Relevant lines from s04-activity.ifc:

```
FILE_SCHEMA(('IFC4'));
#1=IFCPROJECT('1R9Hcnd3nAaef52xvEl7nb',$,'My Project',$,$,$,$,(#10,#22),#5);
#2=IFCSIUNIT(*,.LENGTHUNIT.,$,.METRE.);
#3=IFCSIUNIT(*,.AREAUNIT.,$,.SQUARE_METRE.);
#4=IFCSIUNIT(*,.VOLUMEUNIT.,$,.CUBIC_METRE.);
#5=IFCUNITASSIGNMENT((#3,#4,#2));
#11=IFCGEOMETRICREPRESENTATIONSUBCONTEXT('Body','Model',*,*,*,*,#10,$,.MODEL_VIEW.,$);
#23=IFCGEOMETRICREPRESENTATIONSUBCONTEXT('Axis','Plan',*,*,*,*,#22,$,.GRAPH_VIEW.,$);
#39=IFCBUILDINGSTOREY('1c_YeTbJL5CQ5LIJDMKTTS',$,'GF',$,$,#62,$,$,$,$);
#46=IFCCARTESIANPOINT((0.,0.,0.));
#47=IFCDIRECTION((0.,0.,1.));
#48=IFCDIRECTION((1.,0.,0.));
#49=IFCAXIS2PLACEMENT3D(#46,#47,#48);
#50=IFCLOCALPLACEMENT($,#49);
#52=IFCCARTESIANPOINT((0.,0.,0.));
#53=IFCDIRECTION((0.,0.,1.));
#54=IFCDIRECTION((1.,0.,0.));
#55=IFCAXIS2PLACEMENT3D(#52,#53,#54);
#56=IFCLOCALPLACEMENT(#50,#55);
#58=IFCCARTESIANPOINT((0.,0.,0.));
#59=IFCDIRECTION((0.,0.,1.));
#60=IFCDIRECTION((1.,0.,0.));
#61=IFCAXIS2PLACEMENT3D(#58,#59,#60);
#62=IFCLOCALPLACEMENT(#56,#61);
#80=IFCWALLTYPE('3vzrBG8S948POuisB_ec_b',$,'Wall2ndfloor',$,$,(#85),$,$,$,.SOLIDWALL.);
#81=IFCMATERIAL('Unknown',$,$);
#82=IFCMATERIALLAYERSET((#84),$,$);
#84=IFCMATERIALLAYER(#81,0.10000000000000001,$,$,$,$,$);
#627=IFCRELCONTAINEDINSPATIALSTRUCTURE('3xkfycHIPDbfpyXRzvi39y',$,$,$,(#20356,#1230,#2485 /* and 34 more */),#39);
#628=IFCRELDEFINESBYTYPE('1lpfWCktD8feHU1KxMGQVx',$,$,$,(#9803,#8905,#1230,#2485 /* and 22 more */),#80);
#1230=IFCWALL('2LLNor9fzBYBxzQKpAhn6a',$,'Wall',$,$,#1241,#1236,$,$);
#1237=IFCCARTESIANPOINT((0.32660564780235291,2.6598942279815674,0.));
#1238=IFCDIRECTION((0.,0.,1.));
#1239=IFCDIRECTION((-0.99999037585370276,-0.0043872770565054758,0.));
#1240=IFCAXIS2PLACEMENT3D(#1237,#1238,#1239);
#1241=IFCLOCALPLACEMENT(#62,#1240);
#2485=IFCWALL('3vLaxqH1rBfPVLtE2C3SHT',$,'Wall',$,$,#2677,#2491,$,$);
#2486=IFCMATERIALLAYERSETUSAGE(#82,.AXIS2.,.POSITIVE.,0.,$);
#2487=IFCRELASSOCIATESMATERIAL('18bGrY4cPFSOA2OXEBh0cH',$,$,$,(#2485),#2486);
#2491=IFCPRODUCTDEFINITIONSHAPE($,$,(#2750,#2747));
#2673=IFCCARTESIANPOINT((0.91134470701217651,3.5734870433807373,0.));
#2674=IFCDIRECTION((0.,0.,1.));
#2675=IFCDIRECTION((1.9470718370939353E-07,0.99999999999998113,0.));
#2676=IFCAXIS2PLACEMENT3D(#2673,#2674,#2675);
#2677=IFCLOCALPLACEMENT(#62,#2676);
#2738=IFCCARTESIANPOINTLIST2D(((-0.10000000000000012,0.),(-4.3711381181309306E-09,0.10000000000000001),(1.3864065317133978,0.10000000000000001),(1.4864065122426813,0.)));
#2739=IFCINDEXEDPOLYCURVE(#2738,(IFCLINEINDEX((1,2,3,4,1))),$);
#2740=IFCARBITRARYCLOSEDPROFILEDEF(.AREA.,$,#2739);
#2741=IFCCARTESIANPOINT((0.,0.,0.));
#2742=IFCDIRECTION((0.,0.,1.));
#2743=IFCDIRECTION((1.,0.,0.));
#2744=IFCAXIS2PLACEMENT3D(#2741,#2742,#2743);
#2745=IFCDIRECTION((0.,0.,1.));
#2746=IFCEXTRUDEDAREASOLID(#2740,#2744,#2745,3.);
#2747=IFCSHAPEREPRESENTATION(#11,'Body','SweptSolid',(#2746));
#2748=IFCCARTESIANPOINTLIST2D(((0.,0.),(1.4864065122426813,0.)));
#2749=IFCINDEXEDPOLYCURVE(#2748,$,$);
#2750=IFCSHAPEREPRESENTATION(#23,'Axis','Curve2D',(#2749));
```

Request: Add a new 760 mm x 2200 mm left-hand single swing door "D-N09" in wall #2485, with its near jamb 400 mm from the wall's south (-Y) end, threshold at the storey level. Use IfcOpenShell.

```python
import numpy as np
import ifcopenshell
import ifcopenshell.api.feature
import ifcopenshell.api.geometry
import ifcopenshell.api.root
import ifcopenshell.api.spatial
import ifcopenshell.geom
import ifcopenshell.util.element
import ifcopenshell.util.placement
import ifcopenshell.util.representation
import ifcopenshell.util.shape
import ifcopenshell.util.unit

model = ifcopenshell.open("s04-activity.ifc")
unit_scale = ifcopenshell.util.unit.calculate_unit_scale(model)
settings = ifcopenshell.geom.settings()


def volume(element):
    """Net volume in cubic metres, openings subtracted."""
    shape = ifcopenshell.geom.create_shape(settings, element)
    return ifcopenshell.util.shape.get_volume(shape.geometry)


wall = model.by_guid("3vLaxqH1rBfPVLtE2C3SHT")
storey = ifcopenshell.util.element.get_container(wall, ifc_class="IfcBuildingStorey")
context = ifcopenshell.util.representation.get_context(model, "Model", "Body", "MODEL_VIEW")
before = volume(wall)

width, height, from_end, sill = 0.76, 2.2, 0.4, 0.0  # metres

# The wall runs along its own X axis, and the end named is its -X end.
wall_shape = ifcopenshell.geom.create_shape(settings, wall)
x, y, z = ifcopenshell.util.shape.get_vertices(wall_shape.geometry).T
start = x.min() + from_end
face, thickness = float(y.min()), float(y.max() - y.min())
wall_matrix = ifcopenshell.util.placement.get_local_placement(wall.ObjectPlacement)
level = ifcopenshell.util.placement.get_local_placement(storey.ObjectPlacement)[2, 3]


def in_wall(x, y):
    """Placement at x, y metres in the wall's axes, at sill height."""
    matrix = wall_matrix.copy()
    matrix[:, 3] = wall_matrix @ np.array([x / unit_scale, y / unit_scale, 0.0, 1.0])
    matrix[2, 3] = level + sill / unit_scale
    return matrix


# Opening: a box that overshoots both wall faces by 50 mm.
opening = ifcopenshell.api.root.create_entity(model, ifc_class="IfcOpeningElement", predefined_type="OPENING")
box = ifcopenshell.api.geometry.add_wall_representation(
    model, context=context, length=width, height=height, thickness=thickness + 0.1
)
ifcopenshell.api.geometry.assign_representation(model, product=opening, representation=box)
ifcopenshell.api.geometry.edit_object_placement(model, product=opening, matrix=in_wall(start, face - 0.05), is_si=False)
ifcopenshell.api.feature.add_feature(model, feature=opening, element=wall)

door = ifcopenshell.api.root.create_entity(model, ifc_class="IfcDoor", name="D-N09", predefined_type="DOOR")
door.OverallWidth, door.OverallHeight = width / unit_scale, height / unit_scale
door.OperationType = "SINGLE_SWING_LEFT"
body = ifcopenshell.api.geometry.add_door_representation(
    model,
    context=context,
    overall_width=door.OverallWidth,
    overall_height=door.OverallHeight,
    operation_type="SINGLE_SWING_LEFT",
    lining_properties={"LiningDepth": thickness / unit_scale, "ThresholdDepth": thickness / unit_scale},
)
ifcopenshell.api.geometry.assign_representation(model, product=door, representation=body)
ifcopenshell.api.spatial.assign_container(model, products=[door], relating_structure=storey)
ifcopenshell.api.feature.add_filling(model, opening=opening, element=door)

# The lining spans the wall, so the door starts at the wall face.
ifcopenshell.api.geometry.edit_object_placement(model, product=door, matrix=in_wall(start, face), is_si=False)

after = volume(wall)

print(f"wall volume {before:.3f} -> {after:.3f} m3")

model.write("s04-activity-out.ifc")
```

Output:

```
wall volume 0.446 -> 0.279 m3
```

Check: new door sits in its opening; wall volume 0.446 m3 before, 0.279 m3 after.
